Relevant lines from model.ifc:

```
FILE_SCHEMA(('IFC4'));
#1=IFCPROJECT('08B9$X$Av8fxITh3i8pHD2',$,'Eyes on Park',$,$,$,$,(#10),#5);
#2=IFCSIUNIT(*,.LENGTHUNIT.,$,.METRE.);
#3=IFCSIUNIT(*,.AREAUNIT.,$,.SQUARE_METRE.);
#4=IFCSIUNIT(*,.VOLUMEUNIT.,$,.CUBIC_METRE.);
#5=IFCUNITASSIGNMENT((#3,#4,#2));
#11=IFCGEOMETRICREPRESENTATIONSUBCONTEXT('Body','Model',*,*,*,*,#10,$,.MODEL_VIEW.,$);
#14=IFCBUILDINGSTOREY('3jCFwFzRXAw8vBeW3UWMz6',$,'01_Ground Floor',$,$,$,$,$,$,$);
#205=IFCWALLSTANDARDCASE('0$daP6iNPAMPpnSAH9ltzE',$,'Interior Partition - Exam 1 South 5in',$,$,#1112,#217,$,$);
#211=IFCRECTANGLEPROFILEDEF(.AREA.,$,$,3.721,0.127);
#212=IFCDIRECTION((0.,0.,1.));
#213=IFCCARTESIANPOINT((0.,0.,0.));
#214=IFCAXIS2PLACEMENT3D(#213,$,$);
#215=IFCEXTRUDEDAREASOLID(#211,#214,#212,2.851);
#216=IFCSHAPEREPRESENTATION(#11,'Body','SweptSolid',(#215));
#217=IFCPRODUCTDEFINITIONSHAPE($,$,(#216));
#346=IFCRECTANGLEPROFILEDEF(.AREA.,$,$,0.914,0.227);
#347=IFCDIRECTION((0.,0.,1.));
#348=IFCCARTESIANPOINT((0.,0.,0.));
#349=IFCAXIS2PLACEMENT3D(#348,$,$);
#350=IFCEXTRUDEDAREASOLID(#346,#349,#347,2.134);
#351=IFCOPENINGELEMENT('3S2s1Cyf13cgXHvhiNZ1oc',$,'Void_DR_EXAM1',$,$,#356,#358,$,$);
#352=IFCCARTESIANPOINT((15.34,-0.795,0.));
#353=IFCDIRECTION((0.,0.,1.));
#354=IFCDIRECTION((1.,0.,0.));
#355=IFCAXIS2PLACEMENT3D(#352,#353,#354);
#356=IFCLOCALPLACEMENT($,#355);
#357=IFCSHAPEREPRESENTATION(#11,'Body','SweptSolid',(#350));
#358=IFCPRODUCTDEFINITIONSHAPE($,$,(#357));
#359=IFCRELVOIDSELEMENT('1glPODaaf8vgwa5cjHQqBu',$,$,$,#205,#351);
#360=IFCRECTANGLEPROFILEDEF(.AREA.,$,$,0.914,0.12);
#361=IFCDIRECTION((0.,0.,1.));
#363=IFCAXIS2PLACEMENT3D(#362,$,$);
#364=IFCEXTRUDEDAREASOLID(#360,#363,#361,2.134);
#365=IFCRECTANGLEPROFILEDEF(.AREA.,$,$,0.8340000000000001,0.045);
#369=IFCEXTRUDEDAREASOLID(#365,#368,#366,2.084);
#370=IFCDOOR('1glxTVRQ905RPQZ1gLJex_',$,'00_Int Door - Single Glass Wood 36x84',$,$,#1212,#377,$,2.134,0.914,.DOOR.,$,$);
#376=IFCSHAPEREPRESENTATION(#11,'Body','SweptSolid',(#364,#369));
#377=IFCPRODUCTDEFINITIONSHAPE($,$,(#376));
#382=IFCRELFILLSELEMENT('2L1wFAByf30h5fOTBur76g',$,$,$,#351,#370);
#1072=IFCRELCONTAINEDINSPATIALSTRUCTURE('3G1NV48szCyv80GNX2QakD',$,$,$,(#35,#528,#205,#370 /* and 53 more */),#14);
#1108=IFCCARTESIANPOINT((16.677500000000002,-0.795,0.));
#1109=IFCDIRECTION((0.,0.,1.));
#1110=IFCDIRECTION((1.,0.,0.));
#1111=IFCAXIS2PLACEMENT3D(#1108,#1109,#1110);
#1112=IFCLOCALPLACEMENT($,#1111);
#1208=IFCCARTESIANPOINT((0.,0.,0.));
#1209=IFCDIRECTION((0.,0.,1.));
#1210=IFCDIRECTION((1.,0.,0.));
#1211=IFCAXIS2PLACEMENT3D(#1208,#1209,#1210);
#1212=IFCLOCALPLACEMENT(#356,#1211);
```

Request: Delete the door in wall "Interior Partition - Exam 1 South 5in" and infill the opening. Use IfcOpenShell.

```python
import ifcopenshell
import ifcopenshell.api.feature
import ifcopenshell.api.root
import ifcopenshell.geom
import ifcopenshell.util.shape

model = ifcopenshell.open("model.ifc")
settings = ifcopenshell.geom.settings()


def volume(element):
    """Net volume in cubic metres, openings subtracted."""
    shape = ifcopenshell.geom.create_shape(settings, element)
    return ifcopenshell.util.shape.get_volume(shape.geometry)


door = model.by_id(370)
opening = door.FillsVoids[0].RelatingOpeningElement
wall = opening.VoidsElements[0].RelatingBuildingElement
before = volume(wall)

ifcopenshell.api.root.remove_product(model, product=door)
ifcopenshell.api.feature.remove_feature(model, feature=opening)

after = volume(wall)

print(f"wall volume {before:.3f} -> {after:.3f} m3")

model.write("model_edited.ifc")
```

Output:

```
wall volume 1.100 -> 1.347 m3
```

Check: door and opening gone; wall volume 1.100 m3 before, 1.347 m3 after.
